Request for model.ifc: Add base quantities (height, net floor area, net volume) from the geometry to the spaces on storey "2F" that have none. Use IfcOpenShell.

First a look at what the model holds.

```python
import ifcopenshell
import ifcopenshell.util.element
import ifcopenshell.util.unit

model = ifcopenshell.open("model.ifc")
print(model.schema)
for unit_type in ("LENGTHUNIT", "AREAUNIT", "VOLUMEUNIT"):
    print(unit_type, ifcopenshell.util.unit.calculate_unit_scale(model, unit_type))
storey = next(s for s in model.by_type("IfcBuildingStorey") if s.Name == "2F")
spaces = [e for e in ifcopenshell.util.element.get_decomposition(storey) if e.is_a("IfcSpace")]
for e in sorted(spaces, key=lambda e: e.id()):
    print(e.id(), e.is_a(), e.Name, list(ifcopenshell.util.element.get_psets(e, qtos_only=True)), sep=" | ")
```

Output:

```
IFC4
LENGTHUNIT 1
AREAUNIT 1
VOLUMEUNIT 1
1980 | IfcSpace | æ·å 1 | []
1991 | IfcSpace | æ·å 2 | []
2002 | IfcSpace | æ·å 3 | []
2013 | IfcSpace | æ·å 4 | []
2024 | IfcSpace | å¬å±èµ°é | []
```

```python
import ifcopenshell
import ifcopenshell.api.pset
import ifcopenshell.geom
import ifcopenshell.util.element
import ifcopenshell.util.shape
import ifcopenshell.util.unit

model = ifcopenshell.open("model.ifc")
unit_scale = ifcopenshell.util.unit.calculate_unit_scale(model)
area_scale = ifcopenshell.util.unit.calculate_unit_scale(model, "AREAUNIT")
volume_scale = ifcopenshell.util.unit.calculate_unit_scale(model, "VOLUMEUNIT")
settings = ifcopenshell.geom.settings()

storey = next(s for s in model.by_type("IfcBuildingStorey") if s.Name == "2F")
spaces = [e for e in ifcopenshell.util.element.get_decomposition(storey) if e.is_a("IfcSpace")]

for e in sorted(spaces, key=lambda e: e.id()):
    if ifcopenshell.util.element.get_psets(e, qtos_only=True, should_inherit=False):
        continue
    # Geometry comes back in metres, in the element's own axes.
    shape = ifcopenshell.geom.create_shape(settings, e)
    values = {
        "Height": ifcopenshell.util.shape.get_z(shape.geometry) / unit_scale,
        "NetFloorArea": ifcopenshell.util.shape.get_footprint_area(shape.geometry) / area_scale,
        "NetVolume": ifcopenshell.util.shape.get_volume(shape.geometry) / volume_scale,
    }
    qto = ifcopenshell.api.pset.add_qto(model, product=e, name="Qto_SpaceBaseQuantities")
    ifcopenshell.api.pset.edit_qto(model, qto=qto, properties=values)
    print(e.id(), {k: round(v, 3) for k, v in values.items()})

model.write("model_edited.ifc")
```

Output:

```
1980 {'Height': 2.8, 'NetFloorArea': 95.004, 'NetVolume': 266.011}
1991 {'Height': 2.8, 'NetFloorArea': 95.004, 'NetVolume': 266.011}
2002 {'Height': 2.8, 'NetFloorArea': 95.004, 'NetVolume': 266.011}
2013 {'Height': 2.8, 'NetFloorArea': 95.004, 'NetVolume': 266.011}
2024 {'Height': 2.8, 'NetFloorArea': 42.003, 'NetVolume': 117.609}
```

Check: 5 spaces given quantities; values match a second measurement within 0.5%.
